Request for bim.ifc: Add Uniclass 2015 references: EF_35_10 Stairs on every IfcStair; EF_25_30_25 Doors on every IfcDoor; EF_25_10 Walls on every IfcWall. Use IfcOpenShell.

First a look at what the model holds.

```python
import ifcopenshell

model = ifcopenshell.open("bim.ifc")
print(model.schema)
print("classifications:", [c.Name for c in model.by_type("IfcClassification")])
for ifc_class in ("IfcDoor", "IfcRoof", "IfcStair", "IfcWall", "IfcWindow"):
    print(ifc_class, len(model.by_type(ifc_class)))
```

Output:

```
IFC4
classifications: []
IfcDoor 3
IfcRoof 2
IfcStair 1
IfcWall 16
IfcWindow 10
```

```python
import ifcopenshell
import ifcopenshell.api.classification

model = ifcopenshell.open("bim.ifc")

system = ifcopenshell.api.classification.add_classification(model, classification="Uniclass 2015")

codes = {
    "IfcStair": ("EF_35_10", "Stairs"),
    "IfcDoor": ("EF_25_30_25", "Doors"),
    "IfcWall": ("EF_25_10", "Walls"),
}
for ifc_class, (code, name) in codes.items():
    products = model.by_type(ifc_class)
    ifcopenshell.api.classification.add_reference(
        model, products=products, classification=system, identification=code, name=name
    )
    print(code, len(products))

model.write("bim_v2.ifc")
```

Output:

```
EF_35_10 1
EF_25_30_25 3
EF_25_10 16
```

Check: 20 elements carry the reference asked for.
